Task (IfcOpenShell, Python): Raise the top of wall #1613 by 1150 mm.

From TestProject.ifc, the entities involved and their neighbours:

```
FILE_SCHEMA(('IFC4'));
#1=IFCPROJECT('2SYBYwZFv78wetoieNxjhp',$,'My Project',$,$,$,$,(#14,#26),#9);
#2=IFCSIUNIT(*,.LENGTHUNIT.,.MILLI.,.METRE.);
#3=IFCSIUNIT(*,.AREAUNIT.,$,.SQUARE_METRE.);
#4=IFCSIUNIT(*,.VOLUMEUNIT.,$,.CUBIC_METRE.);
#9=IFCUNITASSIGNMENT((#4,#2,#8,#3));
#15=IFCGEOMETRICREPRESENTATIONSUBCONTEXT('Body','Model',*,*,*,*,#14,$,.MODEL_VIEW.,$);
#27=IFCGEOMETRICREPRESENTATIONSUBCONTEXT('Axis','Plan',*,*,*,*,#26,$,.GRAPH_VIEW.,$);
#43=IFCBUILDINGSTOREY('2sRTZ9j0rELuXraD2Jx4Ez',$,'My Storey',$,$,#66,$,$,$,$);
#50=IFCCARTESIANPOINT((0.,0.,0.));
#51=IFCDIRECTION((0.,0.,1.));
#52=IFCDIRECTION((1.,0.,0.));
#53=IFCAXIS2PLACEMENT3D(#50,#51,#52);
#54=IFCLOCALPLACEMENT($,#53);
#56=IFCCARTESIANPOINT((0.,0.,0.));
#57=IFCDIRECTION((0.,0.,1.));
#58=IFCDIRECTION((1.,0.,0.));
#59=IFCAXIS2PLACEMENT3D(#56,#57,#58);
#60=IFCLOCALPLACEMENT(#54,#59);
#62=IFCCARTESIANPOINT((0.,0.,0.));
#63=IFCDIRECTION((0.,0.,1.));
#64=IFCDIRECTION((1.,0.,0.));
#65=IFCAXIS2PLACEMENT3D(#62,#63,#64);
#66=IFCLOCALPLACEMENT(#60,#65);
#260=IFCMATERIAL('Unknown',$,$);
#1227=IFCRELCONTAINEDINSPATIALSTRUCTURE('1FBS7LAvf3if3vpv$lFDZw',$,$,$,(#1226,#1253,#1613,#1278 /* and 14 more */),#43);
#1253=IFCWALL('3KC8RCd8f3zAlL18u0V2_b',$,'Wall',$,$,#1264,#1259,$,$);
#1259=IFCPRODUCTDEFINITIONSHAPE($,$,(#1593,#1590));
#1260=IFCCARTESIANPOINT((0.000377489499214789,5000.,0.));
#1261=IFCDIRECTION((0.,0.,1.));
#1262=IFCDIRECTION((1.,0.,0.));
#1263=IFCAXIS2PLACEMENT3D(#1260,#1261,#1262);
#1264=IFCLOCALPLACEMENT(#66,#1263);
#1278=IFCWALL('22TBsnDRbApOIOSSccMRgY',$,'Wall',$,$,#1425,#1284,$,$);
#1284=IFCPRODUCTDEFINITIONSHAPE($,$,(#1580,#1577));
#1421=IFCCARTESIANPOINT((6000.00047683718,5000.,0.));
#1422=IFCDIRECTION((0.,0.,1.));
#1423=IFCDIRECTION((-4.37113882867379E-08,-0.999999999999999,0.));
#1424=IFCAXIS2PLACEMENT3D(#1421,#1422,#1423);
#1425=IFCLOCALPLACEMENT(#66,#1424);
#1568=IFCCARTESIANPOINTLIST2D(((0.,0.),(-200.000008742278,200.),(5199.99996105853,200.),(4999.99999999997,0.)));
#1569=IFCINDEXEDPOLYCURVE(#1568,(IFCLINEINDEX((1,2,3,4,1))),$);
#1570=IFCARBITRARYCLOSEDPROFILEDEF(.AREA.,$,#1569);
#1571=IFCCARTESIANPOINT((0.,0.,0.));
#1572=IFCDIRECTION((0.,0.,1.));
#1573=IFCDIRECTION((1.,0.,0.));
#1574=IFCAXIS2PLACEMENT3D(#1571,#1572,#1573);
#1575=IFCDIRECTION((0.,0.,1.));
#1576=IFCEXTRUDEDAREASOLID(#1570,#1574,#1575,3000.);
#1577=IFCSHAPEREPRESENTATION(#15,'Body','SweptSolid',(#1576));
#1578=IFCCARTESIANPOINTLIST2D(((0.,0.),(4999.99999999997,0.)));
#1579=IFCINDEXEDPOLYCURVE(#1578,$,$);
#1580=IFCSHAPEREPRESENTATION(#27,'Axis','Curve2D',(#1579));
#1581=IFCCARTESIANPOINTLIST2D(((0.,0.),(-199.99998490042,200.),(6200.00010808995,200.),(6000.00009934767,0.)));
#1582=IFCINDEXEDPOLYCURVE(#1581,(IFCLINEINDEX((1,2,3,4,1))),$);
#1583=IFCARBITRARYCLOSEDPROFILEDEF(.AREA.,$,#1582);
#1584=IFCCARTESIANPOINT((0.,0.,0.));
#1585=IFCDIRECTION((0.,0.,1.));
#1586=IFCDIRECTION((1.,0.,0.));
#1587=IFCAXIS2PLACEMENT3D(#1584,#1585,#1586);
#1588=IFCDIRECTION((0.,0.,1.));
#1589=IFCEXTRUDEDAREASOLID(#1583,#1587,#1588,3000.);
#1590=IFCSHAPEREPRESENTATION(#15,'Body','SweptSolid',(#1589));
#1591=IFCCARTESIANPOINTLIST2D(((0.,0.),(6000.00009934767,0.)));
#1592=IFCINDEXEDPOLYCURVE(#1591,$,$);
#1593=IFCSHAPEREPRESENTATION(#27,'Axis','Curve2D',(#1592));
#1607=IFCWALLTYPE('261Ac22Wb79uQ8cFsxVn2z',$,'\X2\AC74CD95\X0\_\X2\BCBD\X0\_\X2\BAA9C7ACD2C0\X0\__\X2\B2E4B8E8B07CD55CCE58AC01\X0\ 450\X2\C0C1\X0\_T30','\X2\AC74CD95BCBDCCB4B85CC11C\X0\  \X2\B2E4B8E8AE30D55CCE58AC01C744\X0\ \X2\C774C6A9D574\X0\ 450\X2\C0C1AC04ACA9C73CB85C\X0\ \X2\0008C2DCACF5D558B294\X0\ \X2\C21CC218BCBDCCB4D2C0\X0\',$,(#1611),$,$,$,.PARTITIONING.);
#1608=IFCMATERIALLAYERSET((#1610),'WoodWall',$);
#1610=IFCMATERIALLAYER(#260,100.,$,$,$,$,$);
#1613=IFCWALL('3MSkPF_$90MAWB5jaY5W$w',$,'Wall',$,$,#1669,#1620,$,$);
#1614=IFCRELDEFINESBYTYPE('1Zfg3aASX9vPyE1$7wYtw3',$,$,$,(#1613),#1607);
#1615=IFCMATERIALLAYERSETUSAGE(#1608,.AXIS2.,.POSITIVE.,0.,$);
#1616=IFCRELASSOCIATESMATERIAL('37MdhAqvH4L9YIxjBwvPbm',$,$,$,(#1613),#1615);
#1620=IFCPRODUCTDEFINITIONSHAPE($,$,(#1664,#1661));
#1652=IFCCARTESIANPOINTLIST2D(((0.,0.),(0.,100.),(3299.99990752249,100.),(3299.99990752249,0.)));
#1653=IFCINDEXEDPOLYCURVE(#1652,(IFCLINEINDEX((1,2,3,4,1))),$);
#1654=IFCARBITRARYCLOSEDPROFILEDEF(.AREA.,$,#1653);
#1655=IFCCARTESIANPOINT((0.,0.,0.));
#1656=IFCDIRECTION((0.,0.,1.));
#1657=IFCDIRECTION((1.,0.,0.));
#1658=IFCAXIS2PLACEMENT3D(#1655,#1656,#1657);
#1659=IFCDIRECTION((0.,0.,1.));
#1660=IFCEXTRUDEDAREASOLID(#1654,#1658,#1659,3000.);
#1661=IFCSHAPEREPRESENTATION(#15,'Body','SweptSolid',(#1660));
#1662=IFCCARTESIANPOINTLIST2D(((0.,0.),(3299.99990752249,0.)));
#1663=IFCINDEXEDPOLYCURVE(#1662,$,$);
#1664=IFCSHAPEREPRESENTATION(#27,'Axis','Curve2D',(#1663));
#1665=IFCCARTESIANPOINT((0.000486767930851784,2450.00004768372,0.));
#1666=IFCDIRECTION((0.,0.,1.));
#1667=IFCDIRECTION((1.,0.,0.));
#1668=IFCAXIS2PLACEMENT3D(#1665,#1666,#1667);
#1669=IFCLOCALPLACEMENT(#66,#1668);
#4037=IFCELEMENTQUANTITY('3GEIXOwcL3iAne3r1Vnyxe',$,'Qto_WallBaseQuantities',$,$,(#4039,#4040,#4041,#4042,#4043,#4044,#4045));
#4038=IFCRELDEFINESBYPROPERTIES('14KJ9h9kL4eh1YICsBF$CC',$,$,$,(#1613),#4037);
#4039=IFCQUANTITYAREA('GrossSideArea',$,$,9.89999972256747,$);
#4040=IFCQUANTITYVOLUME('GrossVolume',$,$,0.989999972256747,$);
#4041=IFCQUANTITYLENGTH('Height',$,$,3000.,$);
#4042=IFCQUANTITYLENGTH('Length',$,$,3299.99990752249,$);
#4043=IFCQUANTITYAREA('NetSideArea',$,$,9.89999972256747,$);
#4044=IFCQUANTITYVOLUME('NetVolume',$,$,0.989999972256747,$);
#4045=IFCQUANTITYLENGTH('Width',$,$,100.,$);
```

```python
import ifcopenshell
import ifcopenshell.api.pset
import ifcopenshell.geom
import ifcopenshell.util.element
import ifcopenshell.util.representation
import ifcopenshell.util.shape
import ifcopenshell.util.unit

model = ifcopenshell.open("TestProject.ifc")
unit_scale = ifcopenshell.util.unit.calculate_unit_scale(model)
area_scale = ifcopenshell.util.unit.calculate_unit_scale(model, "AREAUNIT")
volume_scale = ifcopenshell.util.unit.calculate_unit_scale(model, "VOLUMEUNIT")
settings = ifcopenshell.geom.settings()


def volume(element):
    """Net volume in cubic metres, openings subtracted."""
    shape = ifcopenshell.geom.create_shape(settings, element)
    return ifcopenshell.util.shape.get_volume(shape.geometry)


wall = model.by_guid("3MSkPF_$90MAWB5jaY5W$w")
before = volume(wall)

body = ifcopenshell.util.representation.get_representation(wall, "Model", "Body")
solid = body.Items[0]
old_height = solid.Depth
solid.Depth += 1.15 / unit_scale
after = volume(wall)
thickness = 0.1  # wall thickness in metres

# Update the stored height, areas and volumes.
qto = model.by_id(ifcopenshell.util.element.get_pset(wall, "Qto_WallBaseQuantities", should_inherit=False)["id"])
ifcopenshell.api.pset.edit_qto(model, qto=qto, properties={
    "GrossSideArea": ifcopenshell.util.element.get_pset(wall, "Qto_WallBaseQuantities", "GrossSideArea") * solid.Depth / old_height,
    "GrossVolume": ifcopenshell.util.element.get_pset(wall, "Qto_WallBaseQuantities", "GrossVolume") * solid.Depth / old_height,
    "Height": solid.Depth,
    "NetSideArea": after / thickness / area_scale,
    "NetVolume": after / volume_scale,
})

print(f"height {old_height:g} -> {solid.Depth:g}, volume {before:.3f} -> {after:.3f} m3")

model.write("TestProject-out.ifc")
```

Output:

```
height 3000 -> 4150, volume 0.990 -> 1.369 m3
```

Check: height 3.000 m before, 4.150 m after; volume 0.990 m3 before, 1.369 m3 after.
